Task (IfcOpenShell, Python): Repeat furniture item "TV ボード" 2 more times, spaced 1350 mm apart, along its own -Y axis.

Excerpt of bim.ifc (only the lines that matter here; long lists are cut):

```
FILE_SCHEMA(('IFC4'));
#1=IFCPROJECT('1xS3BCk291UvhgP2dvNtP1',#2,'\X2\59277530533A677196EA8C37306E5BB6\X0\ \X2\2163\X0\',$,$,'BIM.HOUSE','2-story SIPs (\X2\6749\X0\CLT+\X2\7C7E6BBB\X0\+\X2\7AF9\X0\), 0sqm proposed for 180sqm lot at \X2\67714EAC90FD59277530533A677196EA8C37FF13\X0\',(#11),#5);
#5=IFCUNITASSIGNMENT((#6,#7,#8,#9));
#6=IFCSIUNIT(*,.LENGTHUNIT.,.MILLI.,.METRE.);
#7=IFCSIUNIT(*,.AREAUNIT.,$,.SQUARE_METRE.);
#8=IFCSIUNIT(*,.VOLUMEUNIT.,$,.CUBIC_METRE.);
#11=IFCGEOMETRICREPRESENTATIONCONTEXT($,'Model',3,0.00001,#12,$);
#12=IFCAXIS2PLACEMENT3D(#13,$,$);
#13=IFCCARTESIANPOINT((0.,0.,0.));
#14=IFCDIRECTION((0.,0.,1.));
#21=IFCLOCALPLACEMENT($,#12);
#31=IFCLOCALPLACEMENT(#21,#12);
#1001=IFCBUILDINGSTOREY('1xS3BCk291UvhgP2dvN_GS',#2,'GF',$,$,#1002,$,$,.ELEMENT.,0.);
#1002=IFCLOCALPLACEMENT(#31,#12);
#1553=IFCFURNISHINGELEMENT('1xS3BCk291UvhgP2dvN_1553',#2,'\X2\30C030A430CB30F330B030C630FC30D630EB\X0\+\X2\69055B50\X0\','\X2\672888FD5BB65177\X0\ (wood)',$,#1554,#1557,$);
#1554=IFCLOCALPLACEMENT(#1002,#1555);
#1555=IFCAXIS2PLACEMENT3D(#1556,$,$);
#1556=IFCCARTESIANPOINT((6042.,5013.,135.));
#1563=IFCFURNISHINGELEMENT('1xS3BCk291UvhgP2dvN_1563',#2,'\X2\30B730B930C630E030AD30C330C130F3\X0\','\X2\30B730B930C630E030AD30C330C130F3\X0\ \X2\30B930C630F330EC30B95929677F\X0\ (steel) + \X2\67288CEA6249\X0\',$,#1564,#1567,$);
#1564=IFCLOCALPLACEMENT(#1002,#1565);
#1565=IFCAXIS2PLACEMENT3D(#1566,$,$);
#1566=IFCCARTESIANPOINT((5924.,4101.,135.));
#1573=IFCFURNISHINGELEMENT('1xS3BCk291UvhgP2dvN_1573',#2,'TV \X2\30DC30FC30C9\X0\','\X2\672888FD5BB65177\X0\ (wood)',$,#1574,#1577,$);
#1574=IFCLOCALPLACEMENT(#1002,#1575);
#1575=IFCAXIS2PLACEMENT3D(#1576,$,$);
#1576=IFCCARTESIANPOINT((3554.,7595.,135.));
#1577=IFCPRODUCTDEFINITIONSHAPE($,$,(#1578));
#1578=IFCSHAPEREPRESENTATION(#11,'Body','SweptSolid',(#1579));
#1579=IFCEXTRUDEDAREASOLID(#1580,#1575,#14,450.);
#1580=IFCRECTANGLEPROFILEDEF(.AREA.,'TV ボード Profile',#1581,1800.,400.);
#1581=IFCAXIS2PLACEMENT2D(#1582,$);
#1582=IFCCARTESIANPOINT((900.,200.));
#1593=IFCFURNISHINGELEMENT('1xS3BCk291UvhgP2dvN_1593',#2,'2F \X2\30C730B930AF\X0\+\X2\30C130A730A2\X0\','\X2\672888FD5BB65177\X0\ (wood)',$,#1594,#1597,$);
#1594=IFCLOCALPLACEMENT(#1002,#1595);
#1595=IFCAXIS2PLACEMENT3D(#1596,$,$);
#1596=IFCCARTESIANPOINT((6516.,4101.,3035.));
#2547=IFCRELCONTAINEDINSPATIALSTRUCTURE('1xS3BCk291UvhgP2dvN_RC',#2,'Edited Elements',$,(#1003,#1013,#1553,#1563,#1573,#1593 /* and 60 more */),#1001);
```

```python
import ifcopenshell
import ifcopenshell.api.geometry
import ifcopenshell.api.root
import ifcopenshell.util.element
import ifcopenshell.util.placement
import ifcopenshell.util.unit

model = ifcopenshell.open("bim.ifc")
unit_scale = ifcopenshell.util.unit.calculate_unit_scale(model)


def reuse_history(source, copy):
    """copy_class also copies each property set's owner history, people and application; keep the originals."""
    for rel in copy.IsDefinedBy:
        if rel.is_a("IfcRelDefinesByProperties") and (history := rel.RelatingPropertyDefinition.OwnerHistory):
            rel.RelatingPropertyDefinition.OwnerHistory = source.OwnerHistory
            ifcopenshell.util.element.remove_deep2(model, history)


source = model.by_id(1573)
base = ifcopenshell.util.placement.get_local_placement(source.ObjectPlacement)
step = -base[:3, 1] * 1.35 / unit_scale

for i in range(1, 3):
    copy = ifcopenshell.api.root.copy_class(model, product=source)
    copy.Representation = ifcopenshell.util.element.copy_deep(
        model, source.Representation, exclude=["IfcGeometricRepresentationContext", "IfcRepresentationMap"]
    )
    reuse_history(source, copy)
    matrix = base.copy()
    matrix[:3, 3] += i * step
    print("added at", matrix[:3, 3].round(3) + 0.0)
    ifcopenshell.api.geometry.edit_object_placement(model, product=copy, matrix=matrix, is_si=False)

model.write("bim_edited.ifc")
```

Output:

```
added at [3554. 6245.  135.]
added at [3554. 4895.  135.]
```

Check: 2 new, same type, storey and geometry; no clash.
